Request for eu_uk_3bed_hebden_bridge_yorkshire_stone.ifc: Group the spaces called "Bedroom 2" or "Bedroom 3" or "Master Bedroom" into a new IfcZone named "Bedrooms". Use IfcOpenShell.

First a look at what the model holds.

```python
import ifcopenshell

model = ifcopenshell.open("eu_uk_3bed_hebden_bridge_yorkshire_stone.ifc")
print(model.schema)
seen = {}
for space in model.by_type("IfcSpace"):
    seen[space.LongName] = seen.get(space.LongName, 0) + 1
for name, count in sorted(seen.items(), key=str):
    print(count, "x", name)
print("zones:", [z.Name for z in model.by_type("IfcZone")][:20])
```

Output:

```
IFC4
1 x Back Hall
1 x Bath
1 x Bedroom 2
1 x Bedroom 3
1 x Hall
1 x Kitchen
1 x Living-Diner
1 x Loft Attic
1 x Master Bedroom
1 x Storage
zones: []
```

```python
import ifcopenshell
import ifcopenshell.api.group
import ifcopenshell.api.root

model = ifcopenshell.open("eu_uk_3bed_hebden_bridge_yorkshire_stone.ifc")

names = {"Bedroom 2", "Bedroom 3", "Master Bedroom"}
spaces = [s for s in model.by_type("IfcSpace") if s.LongName in names]

zone = ifcopenshell.api.root.create_entity(model, ifc_class="IfcZone", name="Bedrooms")
ifcopenshell.api.group.assign_group(model, products=spaces, group=zone)
print(len(spaces), "spaces in", zone.Name)

model.write("eu_uk_3bed_hebden_bridge_yorkshire_stone_rev.ifc")
```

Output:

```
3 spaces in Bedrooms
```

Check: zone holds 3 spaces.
